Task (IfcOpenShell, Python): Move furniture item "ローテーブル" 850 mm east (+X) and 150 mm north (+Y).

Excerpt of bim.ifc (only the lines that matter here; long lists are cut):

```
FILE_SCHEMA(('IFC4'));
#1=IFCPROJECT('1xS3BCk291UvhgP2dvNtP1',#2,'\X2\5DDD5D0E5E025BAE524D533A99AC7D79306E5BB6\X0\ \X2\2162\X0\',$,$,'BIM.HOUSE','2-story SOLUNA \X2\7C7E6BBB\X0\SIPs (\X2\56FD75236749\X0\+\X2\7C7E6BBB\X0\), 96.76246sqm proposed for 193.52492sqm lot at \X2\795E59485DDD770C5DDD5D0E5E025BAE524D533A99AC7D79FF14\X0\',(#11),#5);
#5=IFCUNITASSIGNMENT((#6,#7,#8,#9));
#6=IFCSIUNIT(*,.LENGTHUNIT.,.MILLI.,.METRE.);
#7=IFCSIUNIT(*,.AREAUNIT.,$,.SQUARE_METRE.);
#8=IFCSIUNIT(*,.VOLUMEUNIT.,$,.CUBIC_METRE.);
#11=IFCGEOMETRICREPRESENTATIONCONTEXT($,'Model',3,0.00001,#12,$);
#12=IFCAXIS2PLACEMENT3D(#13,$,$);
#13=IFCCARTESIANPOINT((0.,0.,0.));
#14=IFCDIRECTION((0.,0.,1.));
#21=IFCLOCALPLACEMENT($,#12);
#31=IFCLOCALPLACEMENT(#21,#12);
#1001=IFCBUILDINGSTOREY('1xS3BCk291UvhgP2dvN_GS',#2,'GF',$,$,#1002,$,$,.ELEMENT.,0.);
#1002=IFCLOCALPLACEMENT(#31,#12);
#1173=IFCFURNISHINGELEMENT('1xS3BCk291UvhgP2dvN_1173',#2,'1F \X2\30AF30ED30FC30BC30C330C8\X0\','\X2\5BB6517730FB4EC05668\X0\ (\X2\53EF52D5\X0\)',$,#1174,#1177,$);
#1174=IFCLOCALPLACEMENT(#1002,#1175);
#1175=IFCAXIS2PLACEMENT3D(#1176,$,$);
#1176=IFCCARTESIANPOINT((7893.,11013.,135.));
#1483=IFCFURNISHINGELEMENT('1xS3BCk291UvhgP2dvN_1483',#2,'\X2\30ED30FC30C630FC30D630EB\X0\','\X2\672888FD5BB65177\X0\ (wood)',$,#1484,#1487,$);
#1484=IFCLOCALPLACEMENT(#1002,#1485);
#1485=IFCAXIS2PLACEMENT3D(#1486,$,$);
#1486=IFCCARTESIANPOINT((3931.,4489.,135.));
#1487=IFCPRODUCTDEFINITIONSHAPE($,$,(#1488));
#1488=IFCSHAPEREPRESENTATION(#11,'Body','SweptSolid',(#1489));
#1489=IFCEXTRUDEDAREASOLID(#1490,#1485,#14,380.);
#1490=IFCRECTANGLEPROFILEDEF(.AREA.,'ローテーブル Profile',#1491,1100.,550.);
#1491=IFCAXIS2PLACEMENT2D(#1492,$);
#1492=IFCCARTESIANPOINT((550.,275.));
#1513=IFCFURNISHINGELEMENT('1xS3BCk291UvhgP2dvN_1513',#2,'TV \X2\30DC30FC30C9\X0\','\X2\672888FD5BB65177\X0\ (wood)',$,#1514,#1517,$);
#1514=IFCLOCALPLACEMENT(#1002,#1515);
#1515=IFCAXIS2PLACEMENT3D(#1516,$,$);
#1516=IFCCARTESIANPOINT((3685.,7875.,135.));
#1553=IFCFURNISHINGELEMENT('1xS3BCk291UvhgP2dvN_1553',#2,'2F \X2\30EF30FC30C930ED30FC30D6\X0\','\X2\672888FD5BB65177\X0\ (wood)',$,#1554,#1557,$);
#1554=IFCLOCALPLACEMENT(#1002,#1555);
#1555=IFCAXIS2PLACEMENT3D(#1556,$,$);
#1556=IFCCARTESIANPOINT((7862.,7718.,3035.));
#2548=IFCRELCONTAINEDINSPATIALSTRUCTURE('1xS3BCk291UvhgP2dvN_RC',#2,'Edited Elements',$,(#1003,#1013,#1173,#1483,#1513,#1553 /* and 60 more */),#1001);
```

```python
import ifcopenshell
import ifcopenshell.api.geometry
import ifcopenshell.util.placement

model = ifcopenshell.open("bim.ifc")

item = model.by_id(1483)
matrix = ifcopenshell.util.placement.get_local_placement(item.ObjectPlacement)
matrix[0, 3] += 850.0
matrix[1, 3] += 150.0
ifcopenshell.api.geometry.edit_object_placement(model, product=item, matrix=matrix, is_si=False)

print(ifcopenshell.util.placement.get_local_placement(item.ObjectPlacement).round(3) + 0.0)

model.write("bim_edited.ifc")
```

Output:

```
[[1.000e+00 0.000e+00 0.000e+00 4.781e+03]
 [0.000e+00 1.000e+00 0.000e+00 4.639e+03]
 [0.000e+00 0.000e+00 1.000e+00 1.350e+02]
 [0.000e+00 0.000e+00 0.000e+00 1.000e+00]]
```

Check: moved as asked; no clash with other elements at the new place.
